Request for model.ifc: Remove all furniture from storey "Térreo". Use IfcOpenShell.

First a look at what the model holds.

```python
import ifcopenshell
import ifcopenshell.util.element

model = ifcopenshell.open("model.ifc")
print(model.schema)
storey = next(s for s in model.by_type("IfcBuildingStorey") if s.Name == "Térreo")
furniture = [e for e in ifcopenshell.util.element.get_decomposition(storey) if e.is_a("IfcFurnishingElement")]
seen = {}
for e in furniture:
    element_type = ifcopenshell.util.element.get_type(e)
    name = element_type.Name if element_type not in (None, e) else None
    seen[name] = seen.get(name, 0) + 1
for name, count in sorted(seen.items(), key=str):
    print(count, "x", name)
```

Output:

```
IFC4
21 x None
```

```python
import ifcopenshell
import ifcopenshell.api.root
import ifcopenshell.util.element

model = ifcopenshell.open("model.ifc")

storey = next(s for s in model.by_type("IfcBuildingStorey") if s.Name == "Térreo")
furniture = [e for e in ifcopenshell.util.element.get_decomposition(storey) if e.is_a("IfcFurnishingElement")]

for e in furniture:
    ifcopenshell.api.root.remove_product(model, product=e)
print(len(furniture), "removed")

model.write("model_rev.ifc")
```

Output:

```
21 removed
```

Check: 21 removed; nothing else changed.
